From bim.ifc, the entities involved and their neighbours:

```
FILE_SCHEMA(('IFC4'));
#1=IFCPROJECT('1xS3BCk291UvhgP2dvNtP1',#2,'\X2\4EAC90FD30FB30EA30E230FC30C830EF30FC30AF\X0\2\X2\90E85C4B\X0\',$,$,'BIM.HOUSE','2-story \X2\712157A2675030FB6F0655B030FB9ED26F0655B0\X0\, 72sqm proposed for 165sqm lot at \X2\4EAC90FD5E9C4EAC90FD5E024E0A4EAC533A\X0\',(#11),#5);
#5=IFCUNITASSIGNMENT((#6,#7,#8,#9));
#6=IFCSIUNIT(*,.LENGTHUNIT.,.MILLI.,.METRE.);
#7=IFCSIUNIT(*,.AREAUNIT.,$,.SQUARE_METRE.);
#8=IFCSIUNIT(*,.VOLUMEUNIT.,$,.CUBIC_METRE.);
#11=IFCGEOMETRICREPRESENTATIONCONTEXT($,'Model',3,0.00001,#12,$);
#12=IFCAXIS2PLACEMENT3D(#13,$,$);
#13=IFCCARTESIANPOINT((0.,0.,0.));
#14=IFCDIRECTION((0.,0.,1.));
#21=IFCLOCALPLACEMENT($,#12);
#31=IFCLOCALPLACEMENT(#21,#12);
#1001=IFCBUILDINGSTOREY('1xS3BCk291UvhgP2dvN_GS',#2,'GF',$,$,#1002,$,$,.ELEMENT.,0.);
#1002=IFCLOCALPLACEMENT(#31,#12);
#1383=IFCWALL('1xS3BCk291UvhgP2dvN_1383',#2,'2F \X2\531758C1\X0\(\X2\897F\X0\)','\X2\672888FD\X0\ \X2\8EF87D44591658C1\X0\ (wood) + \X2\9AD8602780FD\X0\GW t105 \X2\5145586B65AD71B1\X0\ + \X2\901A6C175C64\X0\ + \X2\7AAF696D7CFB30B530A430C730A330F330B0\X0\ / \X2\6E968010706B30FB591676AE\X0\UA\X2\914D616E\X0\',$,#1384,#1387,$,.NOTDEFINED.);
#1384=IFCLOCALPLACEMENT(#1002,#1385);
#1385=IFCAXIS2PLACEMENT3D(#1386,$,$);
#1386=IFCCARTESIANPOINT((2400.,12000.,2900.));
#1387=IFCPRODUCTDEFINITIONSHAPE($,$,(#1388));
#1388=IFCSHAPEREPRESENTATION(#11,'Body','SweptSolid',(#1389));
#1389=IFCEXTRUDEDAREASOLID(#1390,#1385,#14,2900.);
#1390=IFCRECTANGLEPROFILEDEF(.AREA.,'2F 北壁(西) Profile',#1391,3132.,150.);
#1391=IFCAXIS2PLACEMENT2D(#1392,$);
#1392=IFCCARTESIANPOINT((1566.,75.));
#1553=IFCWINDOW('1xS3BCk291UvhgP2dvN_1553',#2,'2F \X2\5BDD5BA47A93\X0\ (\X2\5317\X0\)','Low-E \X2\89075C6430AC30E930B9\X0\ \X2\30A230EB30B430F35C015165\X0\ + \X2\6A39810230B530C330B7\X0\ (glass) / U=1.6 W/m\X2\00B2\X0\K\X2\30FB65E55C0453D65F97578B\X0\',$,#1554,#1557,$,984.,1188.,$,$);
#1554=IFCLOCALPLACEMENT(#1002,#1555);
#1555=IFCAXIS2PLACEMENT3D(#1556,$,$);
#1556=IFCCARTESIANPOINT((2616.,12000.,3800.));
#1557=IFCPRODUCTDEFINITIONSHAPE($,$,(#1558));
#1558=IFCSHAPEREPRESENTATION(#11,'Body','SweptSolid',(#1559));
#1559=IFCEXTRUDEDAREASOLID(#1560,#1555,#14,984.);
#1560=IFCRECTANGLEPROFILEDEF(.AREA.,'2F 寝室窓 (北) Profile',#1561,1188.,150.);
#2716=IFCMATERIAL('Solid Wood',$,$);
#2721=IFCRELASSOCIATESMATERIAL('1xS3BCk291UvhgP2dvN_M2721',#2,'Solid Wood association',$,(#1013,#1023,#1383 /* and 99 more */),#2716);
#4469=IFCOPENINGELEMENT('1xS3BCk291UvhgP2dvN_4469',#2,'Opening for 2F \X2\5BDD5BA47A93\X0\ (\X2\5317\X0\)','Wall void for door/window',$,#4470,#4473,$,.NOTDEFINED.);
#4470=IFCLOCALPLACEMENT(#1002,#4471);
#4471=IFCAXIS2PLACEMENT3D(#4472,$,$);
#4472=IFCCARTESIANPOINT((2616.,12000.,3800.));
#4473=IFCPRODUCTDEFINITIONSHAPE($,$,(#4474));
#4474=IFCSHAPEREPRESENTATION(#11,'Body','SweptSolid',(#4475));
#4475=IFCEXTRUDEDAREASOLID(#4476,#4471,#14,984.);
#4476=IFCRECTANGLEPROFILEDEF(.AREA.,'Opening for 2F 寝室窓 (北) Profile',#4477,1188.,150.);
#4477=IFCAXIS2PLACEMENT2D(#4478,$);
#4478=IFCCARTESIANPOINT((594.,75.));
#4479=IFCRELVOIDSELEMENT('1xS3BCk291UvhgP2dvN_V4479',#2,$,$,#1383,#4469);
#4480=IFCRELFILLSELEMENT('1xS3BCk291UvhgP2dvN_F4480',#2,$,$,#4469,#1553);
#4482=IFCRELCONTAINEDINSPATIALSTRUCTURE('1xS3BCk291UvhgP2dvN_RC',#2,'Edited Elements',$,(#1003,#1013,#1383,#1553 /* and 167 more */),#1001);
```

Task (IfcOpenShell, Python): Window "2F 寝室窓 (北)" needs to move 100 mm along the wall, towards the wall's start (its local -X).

```python
import ifcopenshell
import ifcopenshell.api.geometry
import ifcopenshell.util.placement

model = ifcopenshell.open("bim.ifc")

window = model.by_id(1553)
opening = window.FillsVoids[0].RelatingOpeningElement
wall = opening.VoidsElements[0].RelatingBuildingElement

wall_matrix = ifcopenshell.util.placement.get_local_placement(wall.ObjectPlacement)
shift = wall_matrix[:3, 0] * -100.0
before = ifcopenshell.util.placement.get_local_placement(window.ObjectPlacement)[:3, 3].copy()

# The window is not placed relative to its opening, so move both.
for product in (opening, window):
    matrix = ifcopenshell.util.placement.get_local_placement(product.ObjectPlacement)
    matrix[:3, 3] += shift
    ifcopenshell.api.geometry.edit_object_placement(model, product=product, matrix=matrix, is_si=False)

after = ifcopenshell.util.placement.get_local_placement(window.ObjectPlacement)[:3, 3]
print("window moved by", (after - before).round(3) + 0.0)

model.write("bim_edited.ifc")
```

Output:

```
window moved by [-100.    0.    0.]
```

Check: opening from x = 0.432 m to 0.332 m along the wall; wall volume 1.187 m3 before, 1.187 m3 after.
